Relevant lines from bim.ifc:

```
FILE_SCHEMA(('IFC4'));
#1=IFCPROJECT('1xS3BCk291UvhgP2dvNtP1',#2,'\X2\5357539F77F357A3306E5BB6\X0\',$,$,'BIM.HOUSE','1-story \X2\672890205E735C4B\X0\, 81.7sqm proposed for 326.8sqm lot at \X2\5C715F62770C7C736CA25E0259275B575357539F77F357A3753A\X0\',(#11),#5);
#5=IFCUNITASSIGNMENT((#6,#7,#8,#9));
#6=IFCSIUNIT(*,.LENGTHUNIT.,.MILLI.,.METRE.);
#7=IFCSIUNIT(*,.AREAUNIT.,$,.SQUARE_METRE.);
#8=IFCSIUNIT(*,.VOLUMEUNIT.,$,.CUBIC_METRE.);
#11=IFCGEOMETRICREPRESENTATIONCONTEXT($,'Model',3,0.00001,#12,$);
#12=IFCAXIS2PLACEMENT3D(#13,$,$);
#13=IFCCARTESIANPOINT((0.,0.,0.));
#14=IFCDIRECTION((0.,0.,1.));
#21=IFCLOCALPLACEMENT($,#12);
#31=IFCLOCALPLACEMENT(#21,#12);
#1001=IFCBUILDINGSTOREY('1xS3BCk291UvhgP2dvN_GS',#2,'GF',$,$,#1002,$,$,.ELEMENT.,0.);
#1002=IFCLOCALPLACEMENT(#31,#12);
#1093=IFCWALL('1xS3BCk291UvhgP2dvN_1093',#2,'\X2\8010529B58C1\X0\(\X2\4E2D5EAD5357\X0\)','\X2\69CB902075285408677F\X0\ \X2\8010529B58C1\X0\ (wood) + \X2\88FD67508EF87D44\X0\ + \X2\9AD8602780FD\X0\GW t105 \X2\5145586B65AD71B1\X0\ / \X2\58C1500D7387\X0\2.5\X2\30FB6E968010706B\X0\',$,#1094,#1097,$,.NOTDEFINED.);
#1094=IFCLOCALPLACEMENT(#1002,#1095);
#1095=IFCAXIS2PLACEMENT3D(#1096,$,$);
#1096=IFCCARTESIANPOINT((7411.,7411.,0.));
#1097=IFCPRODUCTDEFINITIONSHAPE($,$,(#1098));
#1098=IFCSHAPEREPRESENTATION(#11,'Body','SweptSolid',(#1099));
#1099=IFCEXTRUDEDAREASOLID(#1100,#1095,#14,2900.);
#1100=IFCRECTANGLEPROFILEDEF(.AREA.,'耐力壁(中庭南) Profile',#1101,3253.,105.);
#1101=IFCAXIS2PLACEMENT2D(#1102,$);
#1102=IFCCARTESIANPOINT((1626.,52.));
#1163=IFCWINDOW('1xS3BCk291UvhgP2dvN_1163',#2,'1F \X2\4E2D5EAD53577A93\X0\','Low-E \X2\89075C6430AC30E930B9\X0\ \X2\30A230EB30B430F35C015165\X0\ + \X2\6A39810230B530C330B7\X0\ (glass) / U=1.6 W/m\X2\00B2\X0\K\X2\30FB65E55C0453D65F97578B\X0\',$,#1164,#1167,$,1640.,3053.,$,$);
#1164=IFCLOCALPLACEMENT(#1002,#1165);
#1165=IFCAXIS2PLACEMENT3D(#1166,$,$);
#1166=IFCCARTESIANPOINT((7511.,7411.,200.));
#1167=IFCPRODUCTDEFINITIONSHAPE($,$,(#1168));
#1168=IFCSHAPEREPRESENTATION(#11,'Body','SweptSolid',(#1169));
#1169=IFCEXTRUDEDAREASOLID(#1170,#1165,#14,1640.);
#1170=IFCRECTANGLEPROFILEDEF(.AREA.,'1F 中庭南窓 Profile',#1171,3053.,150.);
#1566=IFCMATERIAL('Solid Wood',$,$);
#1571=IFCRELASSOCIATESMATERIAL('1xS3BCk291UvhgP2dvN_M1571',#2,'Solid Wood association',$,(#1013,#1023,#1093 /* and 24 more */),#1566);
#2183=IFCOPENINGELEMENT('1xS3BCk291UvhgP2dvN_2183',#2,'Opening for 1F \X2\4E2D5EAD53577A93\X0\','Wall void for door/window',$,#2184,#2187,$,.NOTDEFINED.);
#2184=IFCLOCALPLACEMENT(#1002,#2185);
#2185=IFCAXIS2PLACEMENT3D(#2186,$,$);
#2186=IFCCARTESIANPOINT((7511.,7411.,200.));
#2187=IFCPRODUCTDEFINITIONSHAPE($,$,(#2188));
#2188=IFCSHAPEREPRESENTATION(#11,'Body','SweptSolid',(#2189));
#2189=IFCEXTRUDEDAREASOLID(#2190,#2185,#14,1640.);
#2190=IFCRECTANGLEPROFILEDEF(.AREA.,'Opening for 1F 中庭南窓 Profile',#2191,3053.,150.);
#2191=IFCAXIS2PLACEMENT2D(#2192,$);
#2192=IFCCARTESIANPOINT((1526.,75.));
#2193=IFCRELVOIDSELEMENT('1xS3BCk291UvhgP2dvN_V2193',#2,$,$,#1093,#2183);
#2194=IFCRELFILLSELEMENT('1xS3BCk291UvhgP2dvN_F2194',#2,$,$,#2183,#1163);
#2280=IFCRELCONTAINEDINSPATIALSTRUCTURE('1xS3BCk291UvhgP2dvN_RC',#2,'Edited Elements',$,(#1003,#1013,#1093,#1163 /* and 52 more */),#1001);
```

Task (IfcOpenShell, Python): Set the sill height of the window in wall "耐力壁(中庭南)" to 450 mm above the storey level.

```python
import numpy as np
import ifcopenshell
import ifcopenshell.api.geometry
import ifcopenshell.geom
import ifcopenshell.util.element
import ifcopenshell.util.placement
import ifcopenshell.util.shape
import ifcopenshell.util.unit

model = ifcopenshell.open("bim.ifc")
unit_scale = ifcopenshell.util.unit.calculate_unit_scale(model)

window = model.by_id(1163)
opening = window.FillsVoids[0].RelatingOpeningElement
storey = ifcopenshell.util.element.get_container(window, ifc_class="IfcBuildingStorey")
level = ifcopenshell.util.placement.get_local_placement(storey.ObjectPlacement)[2, 3]

# The opening's origin need not be at the sill, so measure its lowest point.
shape = ifcopenshell.geom.create_shape(ifcopenshell.geom.settings(), opening)
bottom = ifcopenshell.util.shape.get_shape_bottom_elevation(shape, shape.geometry) / unit_scale
dz = level + 0.45 / unit_scale - bottom

shift = np.array([0.0, 0.0, dz])
# The window is not placed relative to its opening, so move both.
for product in (opening, window):
    matrix = ifcopenshell.util.placement.get_local_placement(product.ObjectPlacement)
    matrix[:3, 3] += shift
    ifcopenshell.api.geometry.edit_object_placement(model, product=product, matrix=matrix, is_si=False)

print(f"moved by {dz * unit_scale:+.3f} m")

model.write("bim_rev.ifc")
```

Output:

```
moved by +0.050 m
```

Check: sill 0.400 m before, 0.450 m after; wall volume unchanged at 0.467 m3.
